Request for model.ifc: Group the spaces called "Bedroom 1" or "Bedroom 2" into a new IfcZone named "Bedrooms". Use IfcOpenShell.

First a look at what the model holds.

```python
import ifcopenshell

model = ifcopenshell.open("model.ifc")
print(model.schema)
seen = {}
for space in model.by_type("IfcSpace"):
    seen[space.LongName] = seen.get(space.LongName, 0) + 1
for name, count in sorted(seen.items(), key=str):
    print(count, "x", name)
print("zones:", [z.Name for z in model.by_type("IfcZone")][:20])
```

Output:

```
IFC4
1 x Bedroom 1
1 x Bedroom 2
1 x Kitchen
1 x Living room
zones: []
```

```python
import ifcopenshell
import ifcopenshell.api.group
import ifcopenshell.api.root

model = ifcopenshell.open("model.ifc")

names = {"Bedroom 1", "Bedroom 2"}
spaces = [s for s in model.by_type("IfcSpace") if s.LongName in names]

zone = ifcopenshell.api.root.create_entity(model, ifc_class="IfcZone", name="Bedrooms")
ifcopenshell.api.group.assign_group(model, products=spaces, group=zone)
print(len(spaces), "spaces in", zone.Name)

model.write("model_v2.ifc")
```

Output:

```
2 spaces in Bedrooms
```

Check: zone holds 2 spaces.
